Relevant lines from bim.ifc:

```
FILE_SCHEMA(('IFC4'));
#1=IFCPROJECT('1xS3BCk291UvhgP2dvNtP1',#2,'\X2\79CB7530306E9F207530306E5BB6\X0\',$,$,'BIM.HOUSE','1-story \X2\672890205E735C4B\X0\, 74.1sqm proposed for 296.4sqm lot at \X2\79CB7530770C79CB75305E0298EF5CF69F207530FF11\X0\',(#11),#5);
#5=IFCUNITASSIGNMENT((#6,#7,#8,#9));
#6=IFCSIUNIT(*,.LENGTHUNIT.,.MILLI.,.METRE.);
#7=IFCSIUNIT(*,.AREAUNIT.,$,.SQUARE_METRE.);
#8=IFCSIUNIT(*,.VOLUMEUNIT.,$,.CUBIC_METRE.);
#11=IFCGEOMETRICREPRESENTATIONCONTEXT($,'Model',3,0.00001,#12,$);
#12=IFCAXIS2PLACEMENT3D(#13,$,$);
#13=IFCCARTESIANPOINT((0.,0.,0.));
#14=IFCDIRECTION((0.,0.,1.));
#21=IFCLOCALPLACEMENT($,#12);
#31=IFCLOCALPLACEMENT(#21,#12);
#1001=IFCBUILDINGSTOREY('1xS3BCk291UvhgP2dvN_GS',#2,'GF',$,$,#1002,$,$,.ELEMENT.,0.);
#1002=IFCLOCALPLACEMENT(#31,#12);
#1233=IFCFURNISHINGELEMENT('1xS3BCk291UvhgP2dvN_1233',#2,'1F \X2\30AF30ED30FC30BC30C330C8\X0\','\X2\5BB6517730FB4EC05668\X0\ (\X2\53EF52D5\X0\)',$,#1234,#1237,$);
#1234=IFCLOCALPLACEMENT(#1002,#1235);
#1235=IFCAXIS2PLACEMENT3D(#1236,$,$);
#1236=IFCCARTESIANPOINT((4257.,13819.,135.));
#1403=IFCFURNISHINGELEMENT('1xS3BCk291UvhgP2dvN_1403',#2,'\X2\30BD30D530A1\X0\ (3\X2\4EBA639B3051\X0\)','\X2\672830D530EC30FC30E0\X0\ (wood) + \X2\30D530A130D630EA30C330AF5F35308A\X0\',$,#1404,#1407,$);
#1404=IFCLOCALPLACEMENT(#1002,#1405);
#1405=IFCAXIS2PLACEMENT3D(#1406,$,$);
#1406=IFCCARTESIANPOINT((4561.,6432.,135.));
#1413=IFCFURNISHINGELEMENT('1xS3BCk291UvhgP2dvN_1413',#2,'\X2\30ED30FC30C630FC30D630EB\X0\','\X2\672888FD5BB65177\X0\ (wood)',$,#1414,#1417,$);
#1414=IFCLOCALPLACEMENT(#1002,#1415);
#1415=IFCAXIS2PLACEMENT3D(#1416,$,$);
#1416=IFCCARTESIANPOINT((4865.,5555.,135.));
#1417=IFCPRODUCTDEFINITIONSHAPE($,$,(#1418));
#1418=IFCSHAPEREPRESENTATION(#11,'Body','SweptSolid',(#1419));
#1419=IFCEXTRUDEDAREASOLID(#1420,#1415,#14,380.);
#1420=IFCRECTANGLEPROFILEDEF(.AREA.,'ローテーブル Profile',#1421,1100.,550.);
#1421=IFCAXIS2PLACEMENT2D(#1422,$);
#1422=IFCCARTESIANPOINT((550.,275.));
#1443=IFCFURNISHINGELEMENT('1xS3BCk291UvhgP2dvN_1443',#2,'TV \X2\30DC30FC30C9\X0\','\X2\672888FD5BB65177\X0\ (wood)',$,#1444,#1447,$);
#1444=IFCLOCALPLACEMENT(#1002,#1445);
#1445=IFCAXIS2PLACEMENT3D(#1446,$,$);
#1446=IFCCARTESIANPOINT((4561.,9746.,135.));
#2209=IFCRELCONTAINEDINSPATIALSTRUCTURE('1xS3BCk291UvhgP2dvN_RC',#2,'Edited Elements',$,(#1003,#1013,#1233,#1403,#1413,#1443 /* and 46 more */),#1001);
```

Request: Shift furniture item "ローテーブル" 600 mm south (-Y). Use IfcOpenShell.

```python
import ifcopenshell
import ifcopenshell.api.geometry
import ifcopenshell.util.placement

model = ifcopenshell.open("bim.ifc")

item = model.by_guid("1xS3BCk291UvhgP2dvN_1413")
matrix = ifcopenshell.util.placement.get_local_placement(item.ObjectPlacement)
matrix[1, 3] -= 600.0
ifcopenshell.api.geometry.edit_object_placement(model, product=item, matrix=matrix, is_si=False)

print(ifcopenshell.util.placement.get_local_placement(item.ObjectPlacement).round(3) + 0.0)

model.write("bim_updated.ifc")
```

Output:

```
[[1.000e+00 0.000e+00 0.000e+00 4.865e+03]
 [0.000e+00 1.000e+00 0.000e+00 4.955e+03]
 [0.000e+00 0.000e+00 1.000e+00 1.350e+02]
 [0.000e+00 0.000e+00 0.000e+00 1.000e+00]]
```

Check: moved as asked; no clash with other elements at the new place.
